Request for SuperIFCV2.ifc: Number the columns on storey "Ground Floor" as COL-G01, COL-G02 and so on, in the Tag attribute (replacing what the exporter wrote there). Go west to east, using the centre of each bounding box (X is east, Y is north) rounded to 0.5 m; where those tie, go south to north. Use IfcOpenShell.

First a look at what the model holds.

```python
import ifcopenshell
import ifcopenshell.util.element
import ifcopenshell.util.placement

model = ifcopenshell.open("SuperIFCV2.ifc")
print(model.schema)
storey = next(s for s in model.by_type("IfcBuildingStorey") if s.Name == "Ground Floor")
columns = [e for e in ifcopenshell.util.element.get_decomposition(storey) if e.is_a("IfcColumn")]
for e in sorted(columns, key=lambda e: e.id()):
    origin = ifcopenshell.util.placement.get_local_placement(e.ObjectPlacement)[:3, 3]
    print(e.id(), e.Tag, e.Name, origin.round(2) + 0.0, sep=" | ")
```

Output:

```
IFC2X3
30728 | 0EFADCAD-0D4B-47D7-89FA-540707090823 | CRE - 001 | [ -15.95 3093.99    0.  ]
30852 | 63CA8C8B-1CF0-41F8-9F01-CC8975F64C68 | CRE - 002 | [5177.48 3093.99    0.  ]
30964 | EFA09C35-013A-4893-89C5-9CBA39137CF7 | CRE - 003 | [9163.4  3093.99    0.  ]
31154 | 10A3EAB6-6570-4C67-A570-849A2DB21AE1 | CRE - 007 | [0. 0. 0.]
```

```python
import ifcopenshell
import ifcopenshell.geom
import ifcopenshell.util.element
import ifcopenshell.util.shape

model = ifcopenshell.open("SuperIFCV2.ifc")
settings = ifcopenshell.geom.settings()
settings.set("use-world-coords", True)


def centre(element):
    shape = ifcopenshell.geom.create_shape(settings, element)
    return ifcopenshell.util.shape.get_bbox_centroid(shape.geometry)


storey = next(s for s in model.by_type("IfcBuildingStorey") if s.Name == "Ground Floor")
columns = [e for e in ifcopenshell.util.element.get_decomposition(storey) if e.is_a("IfcColumn")]

# Insertion points can sit at a corner or the storey origin, so sort by the geometry (in metres).
centres = {e: centre(e) for e in columns}
columns.sort(key=lambda e: (round(centres[e][0] / 0.5), centres[e][1]))

for i, e in enumerate(columns, start=1):
    number = f"COL-G{i:02d}"
    e.Tag = number
    print(e.id(), number)

model.write("SuperIFCV2_v2.ifc")
```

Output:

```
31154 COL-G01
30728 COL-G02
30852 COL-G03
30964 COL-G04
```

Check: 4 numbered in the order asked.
